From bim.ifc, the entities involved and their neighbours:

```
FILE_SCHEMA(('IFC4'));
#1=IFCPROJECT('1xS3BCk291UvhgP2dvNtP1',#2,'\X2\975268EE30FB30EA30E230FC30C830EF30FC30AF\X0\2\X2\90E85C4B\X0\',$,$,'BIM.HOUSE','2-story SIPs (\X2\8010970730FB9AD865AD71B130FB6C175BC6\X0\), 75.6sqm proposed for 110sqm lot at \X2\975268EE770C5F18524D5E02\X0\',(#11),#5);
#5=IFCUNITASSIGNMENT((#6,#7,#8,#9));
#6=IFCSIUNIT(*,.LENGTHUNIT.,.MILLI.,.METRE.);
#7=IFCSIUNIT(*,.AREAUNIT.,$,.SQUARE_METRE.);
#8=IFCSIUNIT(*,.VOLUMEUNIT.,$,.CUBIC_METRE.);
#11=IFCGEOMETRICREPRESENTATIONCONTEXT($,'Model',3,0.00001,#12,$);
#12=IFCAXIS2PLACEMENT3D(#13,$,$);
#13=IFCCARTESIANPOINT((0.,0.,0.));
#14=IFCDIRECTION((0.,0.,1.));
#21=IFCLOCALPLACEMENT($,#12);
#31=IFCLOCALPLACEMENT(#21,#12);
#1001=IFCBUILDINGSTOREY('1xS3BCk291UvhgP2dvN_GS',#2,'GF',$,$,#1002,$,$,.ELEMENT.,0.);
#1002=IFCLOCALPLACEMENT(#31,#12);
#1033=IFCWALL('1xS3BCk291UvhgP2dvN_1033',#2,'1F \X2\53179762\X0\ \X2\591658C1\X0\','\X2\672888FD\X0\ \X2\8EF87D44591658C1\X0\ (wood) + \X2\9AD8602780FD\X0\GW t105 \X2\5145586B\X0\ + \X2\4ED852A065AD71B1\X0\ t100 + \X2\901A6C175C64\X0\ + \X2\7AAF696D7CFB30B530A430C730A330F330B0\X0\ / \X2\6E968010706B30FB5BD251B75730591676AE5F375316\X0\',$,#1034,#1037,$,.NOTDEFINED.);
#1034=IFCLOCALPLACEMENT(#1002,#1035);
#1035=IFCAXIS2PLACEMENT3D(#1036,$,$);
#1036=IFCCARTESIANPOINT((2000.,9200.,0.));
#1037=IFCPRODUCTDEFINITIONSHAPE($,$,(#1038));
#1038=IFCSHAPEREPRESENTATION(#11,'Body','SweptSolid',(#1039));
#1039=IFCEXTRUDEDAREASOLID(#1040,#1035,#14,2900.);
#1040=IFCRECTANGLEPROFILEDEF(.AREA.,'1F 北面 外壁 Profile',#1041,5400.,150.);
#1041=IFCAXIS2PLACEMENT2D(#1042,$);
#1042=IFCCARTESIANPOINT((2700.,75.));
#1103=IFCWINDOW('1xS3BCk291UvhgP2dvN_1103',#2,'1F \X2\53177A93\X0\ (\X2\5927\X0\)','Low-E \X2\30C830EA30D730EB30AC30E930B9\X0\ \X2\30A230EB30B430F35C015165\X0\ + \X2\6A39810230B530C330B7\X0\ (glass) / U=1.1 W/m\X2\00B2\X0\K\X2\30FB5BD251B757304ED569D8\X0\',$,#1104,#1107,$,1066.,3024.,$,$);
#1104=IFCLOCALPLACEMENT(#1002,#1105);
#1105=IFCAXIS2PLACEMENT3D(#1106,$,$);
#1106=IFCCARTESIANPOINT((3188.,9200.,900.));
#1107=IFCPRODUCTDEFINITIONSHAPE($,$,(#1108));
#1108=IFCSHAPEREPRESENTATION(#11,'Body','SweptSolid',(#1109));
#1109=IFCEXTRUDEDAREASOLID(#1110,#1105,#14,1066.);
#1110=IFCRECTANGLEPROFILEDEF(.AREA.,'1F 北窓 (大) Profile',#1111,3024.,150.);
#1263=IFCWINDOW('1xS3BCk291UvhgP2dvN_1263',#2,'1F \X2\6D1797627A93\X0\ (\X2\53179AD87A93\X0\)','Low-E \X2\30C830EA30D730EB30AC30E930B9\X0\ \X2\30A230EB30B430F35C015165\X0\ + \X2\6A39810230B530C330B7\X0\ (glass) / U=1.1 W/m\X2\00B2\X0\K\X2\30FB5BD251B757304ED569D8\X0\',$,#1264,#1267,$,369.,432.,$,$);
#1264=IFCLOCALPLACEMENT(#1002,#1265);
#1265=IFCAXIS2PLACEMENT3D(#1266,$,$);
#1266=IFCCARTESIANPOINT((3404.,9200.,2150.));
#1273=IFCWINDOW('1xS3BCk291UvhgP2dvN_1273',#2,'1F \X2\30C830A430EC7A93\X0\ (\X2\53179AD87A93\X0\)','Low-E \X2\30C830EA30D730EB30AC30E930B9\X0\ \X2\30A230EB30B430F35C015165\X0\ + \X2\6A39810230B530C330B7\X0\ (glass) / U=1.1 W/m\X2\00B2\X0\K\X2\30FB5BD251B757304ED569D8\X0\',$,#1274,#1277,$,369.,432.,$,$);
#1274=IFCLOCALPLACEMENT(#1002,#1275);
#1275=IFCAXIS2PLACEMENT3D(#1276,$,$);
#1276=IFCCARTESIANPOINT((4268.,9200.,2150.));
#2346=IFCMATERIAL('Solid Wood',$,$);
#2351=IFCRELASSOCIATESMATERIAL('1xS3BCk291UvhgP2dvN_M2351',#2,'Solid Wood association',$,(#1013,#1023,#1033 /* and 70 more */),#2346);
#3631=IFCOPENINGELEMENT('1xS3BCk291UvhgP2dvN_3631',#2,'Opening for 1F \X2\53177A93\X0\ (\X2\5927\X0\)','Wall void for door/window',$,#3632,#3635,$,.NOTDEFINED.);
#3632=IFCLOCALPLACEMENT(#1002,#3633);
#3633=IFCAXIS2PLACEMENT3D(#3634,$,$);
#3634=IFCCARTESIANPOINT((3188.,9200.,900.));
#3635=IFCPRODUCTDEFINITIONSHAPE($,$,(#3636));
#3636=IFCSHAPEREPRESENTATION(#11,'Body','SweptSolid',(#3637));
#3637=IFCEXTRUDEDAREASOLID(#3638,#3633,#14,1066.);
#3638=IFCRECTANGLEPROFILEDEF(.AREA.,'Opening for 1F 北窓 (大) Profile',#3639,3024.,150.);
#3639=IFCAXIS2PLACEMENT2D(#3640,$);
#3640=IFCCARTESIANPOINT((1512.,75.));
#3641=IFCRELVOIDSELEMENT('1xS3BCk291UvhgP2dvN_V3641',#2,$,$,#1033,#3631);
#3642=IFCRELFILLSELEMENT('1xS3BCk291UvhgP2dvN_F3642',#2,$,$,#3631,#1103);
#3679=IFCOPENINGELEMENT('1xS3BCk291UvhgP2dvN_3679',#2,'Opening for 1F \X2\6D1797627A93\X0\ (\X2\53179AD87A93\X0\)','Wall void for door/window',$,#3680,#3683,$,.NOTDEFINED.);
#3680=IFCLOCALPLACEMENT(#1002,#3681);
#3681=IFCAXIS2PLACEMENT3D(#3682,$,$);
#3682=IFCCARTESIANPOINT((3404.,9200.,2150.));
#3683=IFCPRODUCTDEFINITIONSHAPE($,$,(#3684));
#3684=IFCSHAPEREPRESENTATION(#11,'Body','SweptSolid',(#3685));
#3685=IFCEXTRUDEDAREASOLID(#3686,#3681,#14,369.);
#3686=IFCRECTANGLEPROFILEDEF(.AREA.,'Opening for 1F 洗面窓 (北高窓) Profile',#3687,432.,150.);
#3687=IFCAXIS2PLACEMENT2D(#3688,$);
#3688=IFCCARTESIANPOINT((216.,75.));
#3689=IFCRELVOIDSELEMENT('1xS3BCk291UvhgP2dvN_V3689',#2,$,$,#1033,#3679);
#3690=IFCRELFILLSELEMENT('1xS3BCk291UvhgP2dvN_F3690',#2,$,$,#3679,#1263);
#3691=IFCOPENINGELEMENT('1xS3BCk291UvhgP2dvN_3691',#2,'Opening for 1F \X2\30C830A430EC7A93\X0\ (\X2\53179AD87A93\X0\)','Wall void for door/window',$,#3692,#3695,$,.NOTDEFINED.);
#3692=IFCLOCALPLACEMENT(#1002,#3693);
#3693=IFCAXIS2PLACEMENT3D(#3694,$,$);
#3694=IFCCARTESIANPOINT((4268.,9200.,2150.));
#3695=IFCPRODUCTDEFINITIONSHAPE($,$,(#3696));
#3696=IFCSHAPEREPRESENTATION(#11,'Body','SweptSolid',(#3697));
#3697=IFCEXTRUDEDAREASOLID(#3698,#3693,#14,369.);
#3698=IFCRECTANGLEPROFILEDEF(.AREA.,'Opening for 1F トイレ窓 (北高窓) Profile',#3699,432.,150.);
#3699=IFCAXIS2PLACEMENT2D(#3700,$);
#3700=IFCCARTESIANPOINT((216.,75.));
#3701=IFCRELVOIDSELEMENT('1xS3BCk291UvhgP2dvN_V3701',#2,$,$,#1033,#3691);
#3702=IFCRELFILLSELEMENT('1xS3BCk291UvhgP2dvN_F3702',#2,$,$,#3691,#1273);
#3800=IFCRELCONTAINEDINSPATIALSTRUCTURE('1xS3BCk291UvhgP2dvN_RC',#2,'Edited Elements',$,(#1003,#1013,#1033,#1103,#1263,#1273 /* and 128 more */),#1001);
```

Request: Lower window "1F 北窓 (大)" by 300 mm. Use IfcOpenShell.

```python
import numpy as np
import ifcopenshell
import ifcopenshell.api.geometry
import ifcopenshell.util.placement
import ifcopenshell.util.unit

model = ifcopenshell.open("bim.ifc")
unit_scale = ifcopenshell.util.unit.calculate_unit_scale(model)

window = model.by_guid("1xS3BCk291UvhgP2dvN_1103")
opening = window.FillsVoids[0].RelatingOpeningElement
dz = -300.0

shift = np.array([0.0, 0.0, dz])
# The window is not placed relative to its opening, so move both.
for product in (opening, window):
    matrix = ifcopenshell.util.placement.get_local_placement(product.ObjectPlacement)
    matrix[:3, 3] += shift
    ifcopenshell.api.geometry.edit_object_placement(model, product=product, matrix=matrix, is_si=False)

print(f"moved by {dz * unit_scale:+.3f} m")

model.write("bim_v2.ifc")
```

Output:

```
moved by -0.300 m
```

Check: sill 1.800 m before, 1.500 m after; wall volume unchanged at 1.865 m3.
